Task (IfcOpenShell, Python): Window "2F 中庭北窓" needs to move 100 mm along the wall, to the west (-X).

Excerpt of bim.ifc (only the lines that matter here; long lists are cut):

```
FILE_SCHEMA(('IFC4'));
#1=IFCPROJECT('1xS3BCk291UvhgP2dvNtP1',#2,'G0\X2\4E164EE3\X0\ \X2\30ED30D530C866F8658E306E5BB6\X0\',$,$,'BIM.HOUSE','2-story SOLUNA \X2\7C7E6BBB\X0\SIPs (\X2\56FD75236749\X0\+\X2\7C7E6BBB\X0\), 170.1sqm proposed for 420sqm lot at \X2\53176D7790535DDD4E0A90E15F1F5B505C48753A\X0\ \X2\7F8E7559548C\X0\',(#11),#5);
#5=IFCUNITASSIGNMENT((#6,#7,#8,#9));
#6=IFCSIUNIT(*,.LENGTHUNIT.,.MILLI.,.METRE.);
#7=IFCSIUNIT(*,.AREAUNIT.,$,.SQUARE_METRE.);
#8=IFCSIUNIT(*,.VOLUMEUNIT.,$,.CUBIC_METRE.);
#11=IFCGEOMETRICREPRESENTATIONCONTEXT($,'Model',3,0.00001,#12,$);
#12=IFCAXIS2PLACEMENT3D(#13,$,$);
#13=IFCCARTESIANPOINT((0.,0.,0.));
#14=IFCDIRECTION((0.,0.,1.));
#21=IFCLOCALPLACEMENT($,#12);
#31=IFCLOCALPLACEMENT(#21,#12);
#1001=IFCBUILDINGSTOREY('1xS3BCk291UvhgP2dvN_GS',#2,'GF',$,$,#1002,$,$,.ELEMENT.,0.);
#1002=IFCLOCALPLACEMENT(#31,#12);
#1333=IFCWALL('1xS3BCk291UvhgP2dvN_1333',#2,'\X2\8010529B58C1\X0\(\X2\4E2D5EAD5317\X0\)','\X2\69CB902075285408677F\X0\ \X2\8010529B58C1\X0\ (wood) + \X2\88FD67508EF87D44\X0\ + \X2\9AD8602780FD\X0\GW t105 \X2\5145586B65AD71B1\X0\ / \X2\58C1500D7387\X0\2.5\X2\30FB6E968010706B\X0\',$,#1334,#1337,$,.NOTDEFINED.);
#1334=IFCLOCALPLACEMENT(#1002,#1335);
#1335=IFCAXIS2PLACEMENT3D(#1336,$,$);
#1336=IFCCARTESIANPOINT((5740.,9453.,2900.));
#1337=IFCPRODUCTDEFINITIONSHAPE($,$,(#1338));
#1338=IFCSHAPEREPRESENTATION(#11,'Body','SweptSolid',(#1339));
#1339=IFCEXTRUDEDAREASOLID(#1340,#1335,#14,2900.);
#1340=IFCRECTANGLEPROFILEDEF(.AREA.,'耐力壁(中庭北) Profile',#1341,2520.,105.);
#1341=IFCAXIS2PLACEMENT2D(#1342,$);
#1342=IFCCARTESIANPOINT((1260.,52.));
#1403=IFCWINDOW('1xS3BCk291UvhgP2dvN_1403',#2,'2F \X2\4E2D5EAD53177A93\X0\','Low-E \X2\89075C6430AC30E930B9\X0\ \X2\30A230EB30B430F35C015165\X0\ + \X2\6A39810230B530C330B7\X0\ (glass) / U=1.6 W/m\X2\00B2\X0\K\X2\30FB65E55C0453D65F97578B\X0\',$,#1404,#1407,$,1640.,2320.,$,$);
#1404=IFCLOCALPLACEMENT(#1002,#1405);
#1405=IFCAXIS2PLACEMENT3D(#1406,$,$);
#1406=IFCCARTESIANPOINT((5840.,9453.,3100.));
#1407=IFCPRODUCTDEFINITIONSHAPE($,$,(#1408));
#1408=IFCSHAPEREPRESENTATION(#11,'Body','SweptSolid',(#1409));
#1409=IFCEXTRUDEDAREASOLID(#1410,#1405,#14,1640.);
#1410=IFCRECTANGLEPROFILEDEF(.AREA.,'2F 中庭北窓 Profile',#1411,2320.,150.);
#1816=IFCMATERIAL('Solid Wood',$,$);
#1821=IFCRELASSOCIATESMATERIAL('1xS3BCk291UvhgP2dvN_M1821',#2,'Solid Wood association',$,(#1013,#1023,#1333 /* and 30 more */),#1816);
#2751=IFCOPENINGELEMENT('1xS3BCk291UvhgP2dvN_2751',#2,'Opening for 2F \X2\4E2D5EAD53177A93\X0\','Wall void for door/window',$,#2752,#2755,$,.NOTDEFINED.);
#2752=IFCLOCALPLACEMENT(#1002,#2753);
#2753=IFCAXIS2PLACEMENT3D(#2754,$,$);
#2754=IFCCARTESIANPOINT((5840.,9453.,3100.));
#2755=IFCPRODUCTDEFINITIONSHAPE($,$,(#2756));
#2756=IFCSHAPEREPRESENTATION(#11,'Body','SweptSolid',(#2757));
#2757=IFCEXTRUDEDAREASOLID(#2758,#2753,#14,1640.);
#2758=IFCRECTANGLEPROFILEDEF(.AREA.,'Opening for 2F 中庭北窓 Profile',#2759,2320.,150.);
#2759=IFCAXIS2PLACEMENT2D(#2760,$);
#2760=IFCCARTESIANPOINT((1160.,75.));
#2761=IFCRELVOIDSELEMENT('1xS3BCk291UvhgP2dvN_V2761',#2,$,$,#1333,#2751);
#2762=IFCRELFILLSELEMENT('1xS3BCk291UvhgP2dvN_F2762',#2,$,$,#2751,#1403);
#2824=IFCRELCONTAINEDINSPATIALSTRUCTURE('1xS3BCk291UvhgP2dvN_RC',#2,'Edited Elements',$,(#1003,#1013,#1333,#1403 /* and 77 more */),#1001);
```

```python
import ifcopenshell
import ifcopenshell.api.geometry
import ifcopenshell.util.placement
import ifcopenshell.util.unit

model = ifcopenshell.open("bim.ifc")
unit_scale = ifcopenshell.util.unit.calculate_unit_scale(model)

window = model.by_guid("1xS3BCk291UvhgP2dvN_1403")
opening = window.FillsVoids[0].RelatingOpeningElement
wall = opening.VoidsElements[0].RelatingBuildingElement

wall_matrix = ifcopenshell.util.placement.get_local_placement(wall.ObjectPlacement)
shift = wall_matrix[:3, 0] * -0.1 / unit_scale
before = ifcopenshell.util.placement.get_local_placement(window.ObjectPlacement)[:3, 3].copy()

# The window is not placed relative to its opening, so move both.
for product in (opening, window):
    matrix = ifcopenshell.util.placement.get_local_placement(product.ObjectPlacement)
    matrix[:3, 3] += shift
    ifcopenshell.api.geometry.edit_object_placement(model, product=product, matrix=matrix, is_si=False)

after = ifcopenshell.util.placement.get_local_placement(window.ObjectPlacement)[:3, 3]
print("window moved by", (after - before).round(3) + 0.0)

model.write("bim_edited.ifc")
```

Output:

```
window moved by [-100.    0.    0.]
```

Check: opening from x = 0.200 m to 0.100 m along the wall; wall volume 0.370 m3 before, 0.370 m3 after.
